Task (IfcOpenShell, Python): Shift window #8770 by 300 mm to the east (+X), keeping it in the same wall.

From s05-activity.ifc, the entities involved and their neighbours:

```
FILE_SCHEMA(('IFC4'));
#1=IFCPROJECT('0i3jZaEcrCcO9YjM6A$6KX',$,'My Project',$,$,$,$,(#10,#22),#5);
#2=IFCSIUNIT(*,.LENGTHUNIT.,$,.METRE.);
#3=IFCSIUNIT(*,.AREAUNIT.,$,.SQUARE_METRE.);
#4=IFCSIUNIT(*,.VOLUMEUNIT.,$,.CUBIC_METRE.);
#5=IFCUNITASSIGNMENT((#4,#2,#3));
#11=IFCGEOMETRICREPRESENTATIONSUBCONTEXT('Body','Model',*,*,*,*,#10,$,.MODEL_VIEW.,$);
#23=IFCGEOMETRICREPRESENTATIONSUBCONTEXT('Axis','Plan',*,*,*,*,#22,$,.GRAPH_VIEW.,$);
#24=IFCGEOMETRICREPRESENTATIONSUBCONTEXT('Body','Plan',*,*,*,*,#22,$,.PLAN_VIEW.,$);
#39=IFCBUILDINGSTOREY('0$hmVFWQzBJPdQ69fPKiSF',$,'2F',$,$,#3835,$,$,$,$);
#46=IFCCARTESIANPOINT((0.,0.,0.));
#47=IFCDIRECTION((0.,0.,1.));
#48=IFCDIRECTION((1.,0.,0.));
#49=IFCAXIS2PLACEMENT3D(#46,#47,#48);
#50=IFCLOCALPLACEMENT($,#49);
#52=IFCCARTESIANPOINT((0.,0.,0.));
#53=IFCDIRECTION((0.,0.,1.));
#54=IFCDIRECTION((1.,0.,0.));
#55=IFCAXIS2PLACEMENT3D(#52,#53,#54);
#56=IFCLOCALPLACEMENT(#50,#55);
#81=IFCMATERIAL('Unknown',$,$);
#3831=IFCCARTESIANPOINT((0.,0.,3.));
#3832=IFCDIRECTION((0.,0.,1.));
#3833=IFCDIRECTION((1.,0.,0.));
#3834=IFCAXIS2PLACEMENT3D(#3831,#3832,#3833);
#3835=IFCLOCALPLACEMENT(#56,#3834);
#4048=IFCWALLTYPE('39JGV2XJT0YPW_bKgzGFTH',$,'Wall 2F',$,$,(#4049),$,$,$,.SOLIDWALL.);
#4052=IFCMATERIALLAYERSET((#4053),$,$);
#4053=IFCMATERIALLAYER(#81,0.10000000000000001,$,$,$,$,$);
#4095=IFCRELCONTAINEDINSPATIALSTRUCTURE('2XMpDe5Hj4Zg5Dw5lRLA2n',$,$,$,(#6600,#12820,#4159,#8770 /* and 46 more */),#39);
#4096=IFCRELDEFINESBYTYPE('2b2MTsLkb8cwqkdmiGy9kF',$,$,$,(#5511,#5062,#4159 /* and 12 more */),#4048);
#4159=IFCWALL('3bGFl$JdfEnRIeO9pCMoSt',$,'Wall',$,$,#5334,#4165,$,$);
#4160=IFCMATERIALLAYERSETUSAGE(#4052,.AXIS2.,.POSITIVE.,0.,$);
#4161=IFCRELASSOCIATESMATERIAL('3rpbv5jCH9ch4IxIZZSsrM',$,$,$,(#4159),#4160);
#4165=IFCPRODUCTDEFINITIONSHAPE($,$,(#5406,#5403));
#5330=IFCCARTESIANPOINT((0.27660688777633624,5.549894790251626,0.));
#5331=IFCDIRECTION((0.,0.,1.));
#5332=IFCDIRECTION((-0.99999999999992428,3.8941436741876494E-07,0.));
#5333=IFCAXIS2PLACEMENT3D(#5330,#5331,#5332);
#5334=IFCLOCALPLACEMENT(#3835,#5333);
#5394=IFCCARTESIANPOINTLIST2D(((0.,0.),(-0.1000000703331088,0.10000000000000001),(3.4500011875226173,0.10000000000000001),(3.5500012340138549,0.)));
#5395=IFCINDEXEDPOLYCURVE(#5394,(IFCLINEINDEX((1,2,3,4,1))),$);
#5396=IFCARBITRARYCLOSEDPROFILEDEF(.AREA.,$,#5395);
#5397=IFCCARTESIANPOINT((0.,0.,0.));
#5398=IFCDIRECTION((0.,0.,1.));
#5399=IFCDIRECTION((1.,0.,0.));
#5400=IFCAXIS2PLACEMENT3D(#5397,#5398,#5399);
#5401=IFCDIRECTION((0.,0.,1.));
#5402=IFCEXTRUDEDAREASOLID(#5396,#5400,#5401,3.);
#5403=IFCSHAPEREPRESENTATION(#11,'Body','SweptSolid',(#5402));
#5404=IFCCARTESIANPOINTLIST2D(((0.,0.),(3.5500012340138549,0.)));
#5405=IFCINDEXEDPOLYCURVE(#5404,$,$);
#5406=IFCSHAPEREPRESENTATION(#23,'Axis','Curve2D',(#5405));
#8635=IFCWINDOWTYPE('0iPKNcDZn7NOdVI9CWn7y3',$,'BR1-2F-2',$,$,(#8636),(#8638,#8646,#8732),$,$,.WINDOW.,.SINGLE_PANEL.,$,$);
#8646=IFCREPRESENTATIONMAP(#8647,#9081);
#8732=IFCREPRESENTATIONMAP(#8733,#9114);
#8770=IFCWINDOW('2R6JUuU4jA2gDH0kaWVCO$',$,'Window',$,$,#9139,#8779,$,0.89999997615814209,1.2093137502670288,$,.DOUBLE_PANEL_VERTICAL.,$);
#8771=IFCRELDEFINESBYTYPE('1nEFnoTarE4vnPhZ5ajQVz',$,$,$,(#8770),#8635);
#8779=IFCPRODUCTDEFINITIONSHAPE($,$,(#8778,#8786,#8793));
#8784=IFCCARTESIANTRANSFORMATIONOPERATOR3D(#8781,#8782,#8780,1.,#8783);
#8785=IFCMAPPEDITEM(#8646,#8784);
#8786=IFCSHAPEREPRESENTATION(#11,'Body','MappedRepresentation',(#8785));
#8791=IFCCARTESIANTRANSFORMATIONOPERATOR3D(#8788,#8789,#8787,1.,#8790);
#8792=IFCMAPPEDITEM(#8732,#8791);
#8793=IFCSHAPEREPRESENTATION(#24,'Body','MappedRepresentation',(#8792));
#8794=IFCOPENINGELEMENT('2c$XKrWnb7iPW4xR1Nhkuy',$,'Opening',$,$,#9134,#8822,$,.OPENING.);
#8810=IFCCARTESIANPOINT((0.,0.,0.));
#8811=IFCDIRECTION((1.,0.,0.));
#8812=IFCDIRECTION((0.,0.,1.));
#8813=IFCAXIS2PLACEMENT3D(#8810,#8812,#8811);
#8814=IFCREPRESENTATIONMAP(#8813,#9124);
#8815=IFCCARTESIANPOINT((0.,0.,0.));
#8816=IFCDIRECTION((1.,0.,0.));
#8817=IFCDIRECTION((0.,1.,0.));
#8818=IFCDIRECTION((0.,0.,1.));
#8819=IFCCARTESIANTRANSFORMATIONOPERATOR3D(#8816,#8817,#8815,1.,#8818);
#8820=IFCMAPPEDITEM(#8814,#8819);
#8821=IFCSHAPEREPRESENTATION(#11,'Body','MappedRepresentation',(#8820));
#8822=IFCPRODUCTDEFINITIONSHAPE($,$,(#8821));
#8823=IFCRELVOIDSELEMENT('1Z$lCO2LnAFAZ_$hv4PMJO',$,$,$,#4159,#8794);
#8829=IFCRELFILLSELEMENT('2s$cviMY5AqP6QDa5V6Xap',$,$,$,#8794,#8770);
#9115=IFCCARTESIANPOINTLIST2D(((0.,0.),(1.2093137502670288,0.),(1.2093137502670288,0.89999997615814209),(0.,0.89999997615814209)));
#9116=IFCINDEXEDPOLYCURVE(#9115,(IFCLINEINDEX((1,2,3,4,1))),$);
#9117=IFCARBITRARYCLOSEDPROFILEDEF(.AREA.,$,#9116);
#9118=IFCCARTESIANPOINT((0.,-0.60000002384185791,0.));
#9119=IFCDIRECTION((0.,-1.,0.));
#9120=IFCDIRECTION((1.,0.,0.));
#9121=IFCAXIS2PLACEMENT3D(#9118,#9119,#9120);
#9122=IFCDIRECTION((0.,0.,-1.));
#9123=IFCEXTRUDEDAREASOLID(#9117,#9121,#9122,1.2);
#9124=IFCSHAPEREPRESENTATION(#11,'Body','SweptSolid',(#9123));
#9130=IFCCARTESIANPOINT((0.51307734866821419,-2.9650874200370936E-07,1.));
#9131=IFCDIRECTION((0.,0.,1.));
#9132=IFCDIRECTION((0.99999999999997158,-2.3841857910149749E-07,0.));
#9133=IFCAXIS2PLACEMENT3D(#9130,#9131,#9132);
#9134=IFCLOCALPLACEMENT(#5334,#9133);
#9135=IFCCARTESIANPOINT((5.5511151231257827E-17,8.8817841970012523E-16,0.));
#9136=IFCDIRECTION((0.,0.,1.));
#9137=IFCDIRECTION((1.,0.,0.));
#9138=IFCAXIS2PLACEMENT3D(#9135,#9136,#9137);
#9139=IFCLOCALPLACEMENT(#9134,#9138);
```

```python
import ifcopenshell
import ifcopenshell.api.geometry
import ifcopenshell.util.placement
import ifcopenshell.util.unit

model = ifcopenshell.open("s05-activity.ifc")
unit_scale = ifcopenshell.util.unit.calculate_unit_scale(model)

window = model.by_guid("2R6JUuU4jA2gDH0kaWVCO$")
opening = window.FillsVoids[0].RelatingOpeningElement
wall = opening.VoidsElements[0].RelatingBuildingElement

wall_matrix = ifcopenshell.util.placement.get_local_placement(wall.ObjectPlacement)
shift = wall_matrix[:3, 0] * -0.3 / unit_scale
before = ifcopenshell.util.placement.get_local_placement(window.ObjectPlacement)[:3, 3].copy()

# The window is placed relative to its opening, so it follows when the opening moves.
matrix = ifcopenshell.util.placement.get_local_placement(opening.ObjectPlacement)
matrix[:3, 3] += shift
ifcopenshell.api.geometry.edit_object_placement(
    model, product=opening, matrix=matrix, is_si=False, should_transform_children=True
)

after = ifcopenshell.util.placement.get_local_placement(window.ObjectPlacement)[:3, 3]
print("window moved by", (after - before).round(3) + 0.0)

model.write("s05-activity_edited.ifc")
```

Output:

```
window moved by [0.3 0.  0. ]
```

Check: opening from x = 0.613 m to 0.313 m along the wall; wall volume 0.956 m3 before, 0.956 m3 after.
